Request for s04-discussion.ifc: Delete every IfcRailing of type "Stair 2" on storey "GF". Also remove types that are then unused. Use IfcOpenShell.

First a look at what the model holds.

```python
import ifcopenshell
import ifcopenshell.util.element

model = ifcopenshell.open("s04-discussion.ifc")
print(model.schema)
storey = next(s for s in model.by_type("IfcBuildingStorey") if s.Name == "GF")
railings = [e for e in ifcopenshell.util.element.get_decomposition(storey) if e.is_a("IfcRailing")]
seen = {}
for e in railings:
    element_type = ifcopenshell.util.element.get_type(e)
    name = element_type.Name if element_type not in (None, e) else None
    seen[name] = seen.get(name, 0) + 1
for name, count in sorted(seen.items(), key=str):
    print(count, "x", name)
```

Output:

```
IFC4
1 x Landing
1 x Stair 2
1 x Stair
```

```python
import ifcopenshell
import ifcopenshell.api.root
import ifcopenshell.util.element

model = ifcopenshell.open("s04-discussion.ifc")

storey = next(s for s in model.by_type("IfcBuildingStorey") if s.Name == "GF")
railings = [e for e in ifcopenshell.util.element.get_decomposition(storey) if e.is_a("IfcRailing")]
targets = [e for e in railings if (t := ifcopenshell.util.element.get_type(e)) not in (None, e) and t.Name == "Stair 2"]
types = {ifcopenshell.util.element.get_type(e) for e in targets} - {None, *targets}

for e in targets:
    ifcopenshell.api.root.remove_product(model, product=e)
print(len(targets), "removed")

unused = [t for t in types if not ifcopenshell.util.element.get_types(t)]
for t in unused:
    ifcopenshell.api.root.remove_product(model, product=t)
print(len(unused), "unused types removed")

model.write("s04-discussion_v2.ifc")
```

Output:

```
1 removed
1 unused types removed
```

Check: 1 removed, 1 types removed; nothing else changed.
